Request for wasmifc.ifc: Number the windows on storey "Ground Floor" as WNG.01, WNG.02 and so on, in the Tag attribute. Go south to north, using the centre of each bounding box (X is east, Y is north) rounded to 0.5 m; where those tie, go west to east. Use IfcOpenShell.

First a look at what the model holds.

```python
import ifcopenshell
import ifcopenshell.util.element
import ifcopenshell.util.placement

model = ifcopenshell.open("wasmifc.ifc")
print(model.schema)
storey = next(s for s in model.by_type("IfcBuildingStorey") if s.Name == "Ground Floor")
windows = [e for e in ifcopenshell.util.element.get_decomposition(storey) if e.is_a("IfcWindow")]
for e in sorted(windows, key=lambda e: e.id()):
    origin = ifcopenshell.util.placement.get_local_placement(e.ObjectPlacement)[:3, 3]
    print(e.id(), e.Tag, e.Name, origin.round(2) + 0.0, sep=" | ")
```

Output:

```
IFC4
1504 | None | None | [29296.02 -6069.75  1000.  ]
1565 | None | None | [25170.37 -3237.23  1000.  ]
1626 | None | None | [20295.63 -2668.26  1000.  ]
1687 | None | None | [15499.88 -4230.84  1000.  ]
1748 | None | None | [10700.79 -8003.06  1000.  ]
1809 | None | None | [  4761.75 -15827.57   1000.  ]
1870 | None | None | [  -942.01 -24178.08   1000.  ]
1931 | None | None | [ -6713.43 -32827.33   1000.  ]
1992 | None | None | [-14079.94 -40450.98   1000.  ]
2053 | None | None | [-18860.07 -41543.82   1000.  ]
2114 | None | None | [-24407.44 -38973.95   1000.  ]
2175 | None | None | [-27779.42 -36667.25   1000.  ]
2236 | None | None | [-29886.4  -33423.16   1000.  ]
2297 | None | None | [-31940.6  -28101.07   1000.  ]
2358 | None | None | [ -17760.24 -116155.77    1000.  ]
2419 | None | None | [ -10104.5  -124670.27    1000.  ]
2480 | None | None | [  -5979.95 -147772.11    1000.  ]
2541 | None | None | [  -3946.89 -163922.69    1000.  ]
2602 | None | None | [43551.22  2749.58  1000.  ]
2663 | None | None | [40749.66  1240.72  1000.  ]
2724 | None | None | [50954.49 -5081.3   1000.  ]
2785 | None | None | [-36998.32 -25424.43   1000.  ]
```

```python
import ifcopenshell
import ifcopenshell.geom
import ifcopenshell.util.element
import ifcopenshell.util.shape

model = ifcopenshell.open("wasmifc.ifc")
settings = ifcopenshell.geom.settings()
settings.set("use-world-coords", True)


def centre(element):
    shape = ifcopenshell.geom.create_shape(settings, element)
    return ifcopenshell.util.shape.get_bbox_centroid(shape.geometry)


storey = next(s for s in model.by_type("IfcBuildingStorey") if s.Name == "Ground Floor")
windows = [e for e in ifcopenshell.util.element.get_decomposition(storey) if e.is_a("IfcWindow")]

# Insertion points can sit at a corner or the storey origin, so sort by the geometry (in metres).
centres = {e: centre(e) for e in windows}
windows.sort(key=lambda e: (round(centres[e][1] / 0.5), centres[e][0]))

for i, e in enumerate(windows, start=1):
    number = f"WNG.{i:02d}"
    e.Tag = number
    print(e.id(), number)

model.write("wasmifc_edited.ifc")
```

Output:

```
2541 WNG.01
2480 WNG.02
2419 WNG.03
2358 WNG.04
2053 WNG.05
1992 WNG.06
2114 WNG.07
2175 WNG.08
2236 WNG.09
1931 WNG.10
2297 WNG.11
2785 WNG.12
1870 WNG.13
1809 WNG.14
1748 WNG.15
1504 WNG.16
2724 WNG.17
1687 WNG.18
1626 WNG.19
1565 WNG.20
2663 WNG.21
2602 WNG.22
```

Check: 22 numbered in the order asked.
